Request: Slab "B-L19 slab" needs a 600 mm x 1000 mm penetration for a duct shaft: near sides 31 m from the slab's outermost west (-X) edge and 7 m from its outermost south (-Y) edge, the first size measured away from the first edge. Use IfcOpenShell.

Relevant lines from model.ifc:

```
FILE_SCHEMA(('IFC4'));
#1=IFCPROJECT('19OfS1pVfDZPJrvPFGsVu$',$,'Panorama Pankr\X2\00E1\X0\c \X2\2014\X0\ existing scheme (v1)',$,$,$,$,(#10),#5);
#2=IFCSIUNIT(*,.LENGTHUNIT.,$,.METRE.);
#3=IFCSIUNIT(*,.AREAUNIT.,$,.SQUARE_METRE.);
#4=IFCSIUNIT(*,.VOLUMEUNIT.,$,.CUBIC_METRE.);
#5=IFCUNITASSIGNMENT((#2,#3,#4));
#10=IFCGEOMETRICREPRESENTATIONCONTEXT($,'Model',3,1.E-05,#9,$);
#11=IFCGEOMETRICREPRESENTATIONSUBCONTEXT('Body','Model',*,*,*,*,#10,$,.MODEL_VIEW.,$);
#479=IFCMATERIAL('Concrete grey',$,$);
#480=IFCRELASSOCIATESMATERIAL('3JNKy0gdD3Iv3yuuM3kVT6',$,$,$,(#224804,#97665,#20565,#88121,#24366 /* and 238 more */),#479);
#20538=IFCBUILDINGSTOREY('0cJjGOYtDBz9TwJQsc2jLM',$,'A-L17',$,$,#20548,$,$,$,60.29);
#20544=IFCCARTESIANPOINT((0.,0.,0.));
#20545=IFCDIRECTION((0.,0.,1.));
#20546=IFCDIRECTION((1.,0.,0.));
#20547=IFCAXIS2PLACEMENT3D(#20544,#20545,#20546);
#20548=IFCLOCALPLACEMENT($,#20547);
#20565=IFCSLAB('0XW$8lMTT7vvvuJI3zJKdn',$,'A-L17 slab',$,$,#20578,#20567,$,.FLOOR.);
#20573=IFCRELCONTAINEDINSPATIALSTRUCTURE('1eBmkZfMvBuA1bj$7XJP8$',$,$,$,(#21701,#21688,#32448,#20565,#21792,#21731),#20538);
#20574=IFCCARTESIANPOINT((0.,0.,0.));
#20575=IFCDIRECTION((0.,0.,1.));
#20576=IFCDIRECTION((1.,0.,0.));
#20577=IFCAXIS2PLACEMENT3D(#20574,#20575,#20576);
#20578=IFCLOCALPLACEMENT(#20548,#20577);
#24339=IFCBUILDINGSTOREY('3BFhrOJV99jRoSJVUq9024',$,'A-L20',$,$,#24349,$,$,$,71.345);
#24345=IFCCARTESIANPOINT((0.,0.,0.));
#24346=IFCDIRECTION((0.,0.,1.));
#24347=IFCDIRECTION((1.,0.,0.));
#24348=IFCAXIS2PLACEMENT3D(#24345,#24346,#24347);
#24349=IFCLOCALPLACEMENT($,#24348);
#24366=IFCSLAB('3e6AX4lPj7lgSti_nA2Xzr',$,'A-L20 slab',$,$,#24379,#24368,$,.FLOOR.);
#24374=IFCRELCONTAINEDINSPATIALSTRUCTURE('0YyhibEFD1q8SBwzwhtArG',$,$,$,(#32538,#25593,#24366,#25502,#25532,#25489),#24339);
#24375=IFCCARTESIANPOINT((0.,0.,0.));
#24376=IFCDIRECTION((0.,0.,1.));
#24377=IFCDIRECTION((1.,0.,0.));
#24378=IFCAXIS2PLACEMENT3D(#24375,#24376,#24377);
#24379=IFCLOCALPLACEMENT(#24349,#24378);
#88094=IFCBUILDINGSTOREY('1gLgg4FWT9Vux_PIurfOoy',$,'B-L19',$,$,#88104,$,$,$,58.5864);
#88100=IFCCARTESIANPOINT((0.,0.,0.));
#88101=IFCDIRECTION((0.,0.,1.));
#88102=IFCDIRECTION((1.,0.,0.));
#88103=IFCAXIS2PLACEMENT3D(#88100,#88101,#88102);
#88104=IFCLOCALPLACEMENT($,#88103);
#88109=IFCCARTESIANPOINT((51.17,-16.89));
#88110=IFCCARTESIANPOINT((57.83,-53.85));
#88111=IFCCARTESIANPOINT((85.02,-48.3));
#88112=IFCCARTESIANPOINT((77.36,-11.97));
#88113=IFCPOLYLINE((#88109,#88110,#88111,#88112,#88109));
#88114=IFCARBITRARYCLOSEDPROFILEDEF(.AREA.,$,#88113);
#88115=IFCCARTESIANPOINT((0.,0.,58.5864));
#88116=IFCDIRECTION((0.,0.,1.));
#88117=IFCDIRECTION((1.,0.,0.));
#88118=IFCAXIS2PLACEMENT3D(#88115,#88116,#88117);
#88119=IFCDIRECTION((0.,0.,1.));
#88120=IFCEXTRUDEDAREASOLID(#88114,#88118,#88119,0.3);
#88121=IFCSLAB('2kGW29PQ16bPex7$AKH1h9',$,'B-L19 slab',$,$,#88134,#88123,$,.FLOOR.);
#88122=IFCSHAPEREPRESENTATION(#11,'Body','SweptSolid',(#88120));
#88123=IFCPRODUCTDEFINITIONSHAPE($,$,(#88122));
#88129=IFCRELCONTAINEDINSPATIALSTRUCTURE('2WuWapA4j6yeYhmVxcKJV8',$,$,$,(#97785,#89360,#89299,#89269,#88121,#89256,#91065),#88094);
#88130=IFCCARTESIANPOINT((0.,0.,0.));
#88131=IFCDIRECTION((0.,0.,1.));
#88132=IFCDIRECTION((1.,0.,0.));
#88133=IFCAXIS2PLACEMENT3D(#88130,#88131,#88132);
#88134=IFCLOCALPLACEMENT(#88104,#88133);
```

```python
import numpy as np
import ifcopenshell
import ifcopenshell.api.feature
import ifcopenshell.api.geometry
import ifcopenshell.api.root
import ifcopenshell.geom
import ifcopenshell.util.placement
import ifcopenshell.util.representation
import ifcopenshell.util.shape
import ifcopenshell.util.unit

model = ifcopenshell.open("model.ifc")
unit_scale = ifcopenshell.util.unit.calculate_unit_scale(model)
settings = ifcopenshell.geom.settings()


def volume(element):
    """Net volume in cubic metres, openings subtracted."""
    shape = ifcopenshell.geom.create_shape(settings, element)
    return ifcopenshell.util.shape.get_volume(shape.geometry)


slab = model.by_guid("2kGW29PQ16bPex7$AKH1h9")
before = volume(slab)

# Extent in the slab's own axes, in metres. The edges named are its -X and -Y sides.
slab_shape = ifcopenshell.geom.create_shape(settings, slab)
vertices = ifcopenshell.util.shape.get_vertices(slab_shape.geometry)
x_min, y_min, bottom = vertices.min(axis=0)
top = vertices[:, 2].max()

opening = ifcopenshell.api.root.create_entity(model, ifc_class="IfcOpeningElement", name="Duct shaft opening", predefined_type="OPENING")
context = ifcopenshell.util.representation.get_context(model, "Model", "Body", "MODEL_VIEW")
width, depth = 0.6, 1
outline = [(0.0, 0.0), (width, 0.0), (width, depth), (0.0, depth), (0.0, 0.0)]
# Overshoot both faces by 50 mm so the cut is clean.
shape = ifcopenshell.api.geometry.add_slab_representation(
    model, context=context, depth=top - bottom + 0.1, polyline=outline
)
ifcopenshell.api.geometry.assign_representation(model, product=opening, representation=shape)

matrix = ifcopenshell.util.placement.get_local_placement(slab.ObjectPlacement)
matrix[:, 3] = matrix @ np.append(np.array([x_min + 31, y_min + 7, bottom - 0.05]) / unit_scale, 1.0)
ifcopenshell.api.geometry.edit_object_placement(model, product=opening, matrix=matrix, is_si=False)
ifcopenshell.api.feature.add_feature(model, feature=opening, element=slab)

after = volume(slab)

print(f"slab volume {before:.3f} -> {after:.3f} m3")

model.write("model_v2.ifc")
```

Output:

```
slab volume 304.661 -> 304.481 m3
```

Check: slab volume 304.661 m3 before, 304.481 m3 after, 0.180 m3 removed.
